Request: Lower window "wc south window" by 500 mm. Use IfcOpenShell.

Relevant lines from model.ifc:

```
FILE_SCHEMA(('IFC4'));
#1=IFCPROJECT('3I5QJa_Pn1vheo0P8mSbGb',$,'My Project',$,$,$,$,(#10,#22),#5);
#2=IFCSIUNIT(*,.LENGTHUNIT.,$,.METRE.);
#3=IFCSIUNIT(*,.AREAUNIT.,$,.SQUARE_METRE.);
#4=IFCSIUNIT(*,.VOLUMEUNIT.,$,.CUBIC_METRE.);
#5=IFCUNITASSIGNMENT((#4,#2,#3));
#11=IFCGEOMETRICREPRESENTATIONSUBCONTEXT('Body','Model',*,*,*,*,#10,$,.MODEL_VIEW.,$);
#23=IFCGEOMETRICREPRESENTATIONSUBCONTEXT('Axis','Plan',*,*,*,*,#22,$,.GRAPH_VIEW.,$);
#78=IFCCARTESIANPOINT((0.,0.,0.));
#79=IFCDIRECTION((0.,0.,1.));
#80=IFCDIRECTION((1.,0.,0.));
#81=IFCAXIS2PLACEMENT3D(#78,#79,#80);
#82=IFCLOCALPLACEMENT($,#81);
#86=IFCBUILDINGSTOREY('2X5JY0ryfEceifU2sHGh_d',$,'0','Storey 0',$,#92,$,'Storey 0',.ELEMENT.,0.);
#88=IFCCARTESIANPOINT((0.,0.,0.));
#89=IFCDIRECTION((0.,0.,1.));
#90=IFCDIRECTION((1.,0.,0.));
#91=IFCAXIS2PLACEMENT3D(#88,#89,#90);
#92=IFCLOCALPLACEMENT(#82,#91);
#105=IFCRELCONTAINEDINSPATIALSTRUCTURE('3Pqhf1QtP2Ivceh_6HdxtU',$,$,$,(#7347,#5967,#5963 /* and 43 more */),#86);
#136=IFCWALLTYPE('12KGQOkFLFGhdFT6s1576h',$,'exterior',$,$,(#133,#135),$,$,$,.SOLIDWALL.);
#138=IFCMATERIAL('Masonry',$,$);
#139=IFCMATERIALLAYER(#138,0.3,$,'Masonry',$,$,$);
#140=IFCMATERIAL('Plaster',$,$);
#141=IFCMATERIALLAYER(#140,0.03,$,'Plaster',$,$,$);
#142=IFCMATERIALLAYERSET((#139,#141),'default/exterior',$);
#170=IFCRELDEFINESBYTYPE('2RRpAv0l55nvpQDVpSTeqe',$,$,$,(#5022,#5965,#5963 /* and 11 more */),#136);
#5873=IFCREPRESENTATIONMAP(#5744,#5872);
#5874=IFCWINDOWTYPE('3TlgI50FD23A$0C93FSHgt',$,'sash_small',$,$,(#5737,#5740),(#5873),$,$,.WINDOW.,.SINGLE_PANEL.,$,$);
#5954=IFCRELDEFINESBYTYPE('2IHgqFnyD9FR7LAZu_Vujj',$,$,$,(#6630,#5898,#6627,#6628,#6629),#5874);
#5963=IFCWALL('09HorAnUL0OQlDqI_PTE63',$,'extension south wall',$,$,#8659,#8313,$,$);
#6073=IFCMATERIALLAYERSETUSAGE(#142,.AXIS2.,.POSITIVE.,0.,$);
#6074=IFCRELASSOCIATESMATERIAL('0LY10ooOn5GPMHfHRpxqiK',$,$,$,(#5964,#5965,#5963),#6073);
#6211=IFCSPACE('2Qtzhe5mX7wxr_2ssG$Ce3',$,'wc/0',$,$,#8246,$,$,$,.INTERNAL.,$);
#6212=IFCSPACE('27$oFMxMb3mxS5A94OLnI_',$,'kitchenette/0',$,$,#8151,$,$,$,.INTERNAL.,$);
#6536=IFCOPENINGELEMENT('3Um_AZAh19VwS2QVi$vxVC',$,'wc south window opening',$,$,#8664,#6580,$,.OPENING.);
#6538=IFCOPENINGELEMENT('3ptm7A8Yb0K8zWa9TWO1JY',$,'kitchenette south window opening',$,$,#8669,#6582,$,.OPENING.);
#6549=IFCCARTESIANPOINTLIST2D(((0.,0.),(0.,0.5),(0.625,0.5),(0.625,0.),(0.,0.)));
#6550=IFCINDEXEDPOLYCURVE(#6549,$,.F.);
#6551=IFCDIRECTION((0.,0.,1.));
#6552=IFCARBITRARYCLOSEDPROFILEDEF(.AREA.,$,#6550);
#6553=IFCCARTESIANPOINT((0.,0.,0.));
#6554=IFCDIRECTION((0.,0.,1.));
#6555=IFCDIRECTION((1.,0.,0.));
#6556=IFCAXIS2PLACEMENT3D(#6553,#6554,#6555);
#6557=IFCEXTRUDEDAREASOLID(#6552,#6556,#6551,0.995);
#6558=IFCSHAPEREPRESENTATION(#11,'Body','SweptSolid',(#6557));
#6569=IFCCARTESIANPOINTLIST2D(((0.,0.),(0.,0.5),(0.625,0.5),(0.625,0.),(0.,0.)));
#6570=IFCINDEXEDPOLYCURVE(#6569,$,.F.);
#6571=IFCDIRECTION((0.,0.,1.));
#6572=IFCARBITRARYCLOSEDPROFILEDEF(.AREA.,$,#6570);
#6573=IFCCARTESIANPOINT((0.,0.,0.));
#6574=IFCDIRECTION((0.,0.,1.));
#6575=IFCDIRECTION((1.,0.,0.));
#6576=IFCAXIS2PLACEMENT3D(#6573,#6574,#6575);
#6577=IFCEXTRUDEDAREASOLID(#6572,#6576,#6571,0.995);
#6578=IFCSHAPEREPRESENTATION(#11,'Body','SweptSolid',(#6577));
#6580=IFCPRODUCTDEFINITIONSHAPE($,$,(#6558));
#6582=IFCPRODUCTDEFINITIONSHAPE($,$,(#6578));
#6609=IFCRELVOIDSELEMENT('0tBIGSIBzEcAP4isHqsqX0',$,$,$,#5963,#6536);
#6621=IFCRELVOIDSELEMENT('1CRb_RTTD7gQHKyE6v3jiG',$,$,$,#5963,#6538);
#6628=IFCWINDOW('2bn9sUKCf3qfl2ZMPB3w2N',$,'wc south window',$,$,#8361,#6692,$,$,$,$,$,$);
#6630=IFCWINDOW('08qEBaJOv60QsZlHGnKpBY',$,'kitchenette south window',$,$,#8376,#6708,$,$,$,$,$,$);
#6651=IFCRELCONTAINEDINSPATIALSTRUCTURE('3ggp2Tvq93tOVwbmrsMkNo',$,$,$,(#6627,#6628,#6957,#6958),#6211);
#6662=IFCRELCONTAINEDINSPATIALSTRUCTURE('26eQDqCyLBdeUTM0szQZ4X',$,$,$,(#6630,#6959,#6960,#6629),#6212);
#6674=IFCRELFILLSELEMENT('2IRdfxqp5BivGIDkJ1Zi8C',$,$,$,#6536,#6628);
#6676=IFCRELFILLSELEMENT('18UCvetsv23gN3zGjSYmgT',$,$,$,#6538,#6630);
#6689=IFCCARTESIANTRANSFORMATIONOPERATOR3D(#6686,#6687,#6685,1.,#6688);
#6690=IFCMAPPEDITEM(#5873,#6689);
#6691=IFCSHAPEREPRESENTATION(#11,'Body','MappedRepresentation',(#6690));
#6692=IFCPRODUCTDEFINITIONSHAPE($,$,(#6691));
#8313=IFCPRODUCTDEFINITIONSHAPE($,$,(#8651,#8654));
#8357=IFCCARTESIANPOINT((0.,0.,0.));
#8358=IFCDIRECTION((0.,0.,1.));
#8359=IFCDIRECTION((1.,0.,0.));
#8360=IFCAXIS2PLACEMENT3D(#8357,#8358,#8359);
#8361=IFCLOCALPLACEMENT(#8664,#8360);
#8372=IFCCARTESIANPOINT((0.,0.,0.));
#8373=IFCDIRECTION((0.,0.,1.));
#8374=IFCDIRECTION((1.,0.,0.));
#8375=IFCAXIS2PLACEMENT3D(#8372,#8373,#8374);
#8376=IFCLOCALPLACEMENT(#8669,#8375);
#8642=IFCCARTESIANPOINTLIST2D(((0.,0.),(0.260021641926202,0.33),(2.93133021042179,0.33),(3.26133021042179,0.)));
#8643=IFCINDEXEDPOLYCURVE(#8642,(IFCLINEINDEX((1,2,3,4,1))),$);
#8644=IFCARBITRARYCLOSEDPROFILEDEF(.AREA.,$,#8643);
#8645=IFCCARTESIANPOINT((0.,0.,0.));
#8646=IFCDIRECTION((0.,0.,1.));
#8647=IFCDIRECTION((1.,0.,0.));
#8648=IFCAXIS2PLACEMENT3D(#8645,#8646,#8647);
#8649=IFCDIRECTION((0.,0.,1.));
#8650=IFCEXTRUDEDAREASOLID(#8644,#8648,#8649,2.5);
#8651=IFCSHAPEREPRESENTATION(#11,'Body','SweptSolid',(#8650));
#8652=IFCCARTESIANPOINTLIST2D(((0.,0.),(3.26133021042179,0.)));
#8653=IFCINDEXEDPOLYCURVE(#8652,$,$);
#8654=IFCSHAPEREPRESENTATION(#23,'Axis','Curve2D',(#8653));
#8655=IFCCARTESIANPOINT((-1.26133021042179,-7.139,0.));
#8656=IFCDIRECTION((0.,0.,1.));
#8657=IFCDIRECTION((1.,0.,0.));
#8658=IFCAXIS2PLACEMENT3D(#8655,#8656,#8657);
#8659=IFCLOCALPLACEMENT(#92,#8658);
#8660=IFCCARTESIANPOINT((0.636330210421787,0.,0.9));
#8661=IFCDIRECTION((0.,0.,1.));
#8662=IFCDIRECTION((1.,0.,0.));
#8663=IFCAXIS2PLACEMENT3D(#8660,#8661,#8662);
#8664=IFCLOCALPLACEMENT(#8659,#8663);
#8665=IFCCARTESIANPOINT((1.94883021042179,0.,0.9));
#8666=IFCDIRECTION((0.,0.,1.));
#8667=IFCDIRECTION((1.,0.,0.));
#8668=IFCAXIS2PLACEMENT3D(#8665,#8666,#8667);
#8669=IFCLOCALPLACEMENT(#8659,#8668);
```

```python
import numpy as np
import ifcopenshell
import ifcopenshell.api.geometry
import ifcopenshell.util.placement
import ifcopenshell.util.unit

model = ifcopenshell.open("model.ifc")
unit_scale = ifcopenshell.util.unit.calculate_unit_scale(model)

window = model.by_id(6628)
opening = window.FillsVoids[0].RelatingOpeningElement
dz = -0.5 / unit_scale

shift = np.array([0.0, 0.0, dz])
# The window is placed relative to its opening, so it follows when the opening moves.
matrix = ifcopenshell.util.placement.get_local_placement(opening.ObjectPlacement)
matrix[:3, 3] += shift
ifcopenshell.api.geometry.edit_object_placement(
    model, product=opening, matrix=matrix, is_si=False, should_transform_children=True
)

print(f"moved by {dz * unit_scale:+.3f} m")

model.write("model-out.ifc")
```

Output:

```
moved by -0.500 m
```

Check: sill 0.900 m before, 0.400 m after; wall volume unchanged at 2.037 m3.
